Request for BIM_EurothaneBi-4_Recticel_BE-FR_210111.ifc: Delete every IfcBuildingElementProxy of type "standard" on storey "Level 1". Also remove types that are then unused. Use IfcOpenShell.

First a look at what the model holds.

```python
import ifcopenshell
import ifcopenshell.util.element

model = ifcopenshell.open("BIM_EurothaneBi-4_Recticel_BE-FR_210111.ifc")
print(model.schema)
storey = next(s for s in model.by_type("IfcBuildingStorey") if s.Name == "Level 1")
proxies = [e for e in ifcopenshell.util.element.get_decomposition(storey) if e.is_a("IfcBuildingElementProxy")]
seen = {}
for e in proxies:
    element_type = ifcopenshell.util.element.get_type(e)
    name = element_type.Name if element_type not in (None, e) else None
    seen[name] = seen.get(name, 0) + 1
for name, count in sorted(seen.items(), key=str):
    print(count, "x", name)
```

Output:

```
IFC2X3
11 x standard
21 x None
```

```python
import ifcopenshell
import ifcopenshell.api.root
import ifcopenshell.util.element

model = ifcopenshell.open("BIM_EurothaneBi-4_Recticel_BE-FR_210111.ifc")

storey = next(s for s in model.by_type("IfcBuildingStorey") if s.Name == "Level 1")
proxies = [e for e in ifcopenshell.util.element.get_decomposition(storey) if e.is_a("IfcBuildingElementProxy")]
targets = [e for e in proxies if (t := ifcopenshell.util.element.get_type(e)) not in (None, e) and t.Name == "standard"]
types = {ifcopenshell.util.element.get_type(e) for e in targets} - {None, *targets}

for e in targets:
    ifcopenshell.api.root.remove_product(model, product=e)
print(len(targets), "removed")

unused = [t for t in types if not ifcopenshell.util.element.get_types(t)]
for t in unused:
    ifcopenshell.api.root.remove_product(model, product=t)
print(len(unused), "unused types removed")

model.write("BIM_EurothaneBi-4_Recticel_BE-FR_210111-out.ifc")
```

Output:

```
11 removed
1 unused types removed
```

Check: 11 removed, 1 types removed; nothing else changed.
